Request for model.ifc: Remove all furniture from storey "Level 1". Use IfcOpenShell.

First a look at what the model holds.

```python
import ifcopenshell
import ifcopenshell.util.element

model = ifcopenshell.open("model.ifc")
print(model.schema)
storey = next(s for s in model.by_type("IfcBuildingStorey") if s.Name == "Level 1")
furniture = [e for e in ifcopenshell.util.element.get_decomposition(storey) if e.is_a("IfcFurnishingElement")]
seen = {}
for e in furniture:
    element_type = ifcopenshell.util.element.get_type(e)
    name = element_type.Name if element_type not in (None, e) else None
    seen[name] = seen.get(name, 0) + 1
for name, count in sorted(seen.items(), key=str):
    print(count, "x", name)
```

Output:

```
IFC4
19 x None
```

```python
import ifcopenshell
import ifcopenshell.api.root
import ifcopenshell.util.element

model = ifcopenshell.open("model.ifc")

storey = next(s for s in model.by_type("IfcBuildingStorey") if s.Name == "Level 1")
furniture = [e for e in ifcopenshell.util.element.get_decomposition(storey) if e.is_a("IfcFurnishingElement")]

for e in furniture:
    ifcopenshell.api.root.remove_product(model, product=e)
print(len(furniture), "removed")

model.write("model-out.ifc")
```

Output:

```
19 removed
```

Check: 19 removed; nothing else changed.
